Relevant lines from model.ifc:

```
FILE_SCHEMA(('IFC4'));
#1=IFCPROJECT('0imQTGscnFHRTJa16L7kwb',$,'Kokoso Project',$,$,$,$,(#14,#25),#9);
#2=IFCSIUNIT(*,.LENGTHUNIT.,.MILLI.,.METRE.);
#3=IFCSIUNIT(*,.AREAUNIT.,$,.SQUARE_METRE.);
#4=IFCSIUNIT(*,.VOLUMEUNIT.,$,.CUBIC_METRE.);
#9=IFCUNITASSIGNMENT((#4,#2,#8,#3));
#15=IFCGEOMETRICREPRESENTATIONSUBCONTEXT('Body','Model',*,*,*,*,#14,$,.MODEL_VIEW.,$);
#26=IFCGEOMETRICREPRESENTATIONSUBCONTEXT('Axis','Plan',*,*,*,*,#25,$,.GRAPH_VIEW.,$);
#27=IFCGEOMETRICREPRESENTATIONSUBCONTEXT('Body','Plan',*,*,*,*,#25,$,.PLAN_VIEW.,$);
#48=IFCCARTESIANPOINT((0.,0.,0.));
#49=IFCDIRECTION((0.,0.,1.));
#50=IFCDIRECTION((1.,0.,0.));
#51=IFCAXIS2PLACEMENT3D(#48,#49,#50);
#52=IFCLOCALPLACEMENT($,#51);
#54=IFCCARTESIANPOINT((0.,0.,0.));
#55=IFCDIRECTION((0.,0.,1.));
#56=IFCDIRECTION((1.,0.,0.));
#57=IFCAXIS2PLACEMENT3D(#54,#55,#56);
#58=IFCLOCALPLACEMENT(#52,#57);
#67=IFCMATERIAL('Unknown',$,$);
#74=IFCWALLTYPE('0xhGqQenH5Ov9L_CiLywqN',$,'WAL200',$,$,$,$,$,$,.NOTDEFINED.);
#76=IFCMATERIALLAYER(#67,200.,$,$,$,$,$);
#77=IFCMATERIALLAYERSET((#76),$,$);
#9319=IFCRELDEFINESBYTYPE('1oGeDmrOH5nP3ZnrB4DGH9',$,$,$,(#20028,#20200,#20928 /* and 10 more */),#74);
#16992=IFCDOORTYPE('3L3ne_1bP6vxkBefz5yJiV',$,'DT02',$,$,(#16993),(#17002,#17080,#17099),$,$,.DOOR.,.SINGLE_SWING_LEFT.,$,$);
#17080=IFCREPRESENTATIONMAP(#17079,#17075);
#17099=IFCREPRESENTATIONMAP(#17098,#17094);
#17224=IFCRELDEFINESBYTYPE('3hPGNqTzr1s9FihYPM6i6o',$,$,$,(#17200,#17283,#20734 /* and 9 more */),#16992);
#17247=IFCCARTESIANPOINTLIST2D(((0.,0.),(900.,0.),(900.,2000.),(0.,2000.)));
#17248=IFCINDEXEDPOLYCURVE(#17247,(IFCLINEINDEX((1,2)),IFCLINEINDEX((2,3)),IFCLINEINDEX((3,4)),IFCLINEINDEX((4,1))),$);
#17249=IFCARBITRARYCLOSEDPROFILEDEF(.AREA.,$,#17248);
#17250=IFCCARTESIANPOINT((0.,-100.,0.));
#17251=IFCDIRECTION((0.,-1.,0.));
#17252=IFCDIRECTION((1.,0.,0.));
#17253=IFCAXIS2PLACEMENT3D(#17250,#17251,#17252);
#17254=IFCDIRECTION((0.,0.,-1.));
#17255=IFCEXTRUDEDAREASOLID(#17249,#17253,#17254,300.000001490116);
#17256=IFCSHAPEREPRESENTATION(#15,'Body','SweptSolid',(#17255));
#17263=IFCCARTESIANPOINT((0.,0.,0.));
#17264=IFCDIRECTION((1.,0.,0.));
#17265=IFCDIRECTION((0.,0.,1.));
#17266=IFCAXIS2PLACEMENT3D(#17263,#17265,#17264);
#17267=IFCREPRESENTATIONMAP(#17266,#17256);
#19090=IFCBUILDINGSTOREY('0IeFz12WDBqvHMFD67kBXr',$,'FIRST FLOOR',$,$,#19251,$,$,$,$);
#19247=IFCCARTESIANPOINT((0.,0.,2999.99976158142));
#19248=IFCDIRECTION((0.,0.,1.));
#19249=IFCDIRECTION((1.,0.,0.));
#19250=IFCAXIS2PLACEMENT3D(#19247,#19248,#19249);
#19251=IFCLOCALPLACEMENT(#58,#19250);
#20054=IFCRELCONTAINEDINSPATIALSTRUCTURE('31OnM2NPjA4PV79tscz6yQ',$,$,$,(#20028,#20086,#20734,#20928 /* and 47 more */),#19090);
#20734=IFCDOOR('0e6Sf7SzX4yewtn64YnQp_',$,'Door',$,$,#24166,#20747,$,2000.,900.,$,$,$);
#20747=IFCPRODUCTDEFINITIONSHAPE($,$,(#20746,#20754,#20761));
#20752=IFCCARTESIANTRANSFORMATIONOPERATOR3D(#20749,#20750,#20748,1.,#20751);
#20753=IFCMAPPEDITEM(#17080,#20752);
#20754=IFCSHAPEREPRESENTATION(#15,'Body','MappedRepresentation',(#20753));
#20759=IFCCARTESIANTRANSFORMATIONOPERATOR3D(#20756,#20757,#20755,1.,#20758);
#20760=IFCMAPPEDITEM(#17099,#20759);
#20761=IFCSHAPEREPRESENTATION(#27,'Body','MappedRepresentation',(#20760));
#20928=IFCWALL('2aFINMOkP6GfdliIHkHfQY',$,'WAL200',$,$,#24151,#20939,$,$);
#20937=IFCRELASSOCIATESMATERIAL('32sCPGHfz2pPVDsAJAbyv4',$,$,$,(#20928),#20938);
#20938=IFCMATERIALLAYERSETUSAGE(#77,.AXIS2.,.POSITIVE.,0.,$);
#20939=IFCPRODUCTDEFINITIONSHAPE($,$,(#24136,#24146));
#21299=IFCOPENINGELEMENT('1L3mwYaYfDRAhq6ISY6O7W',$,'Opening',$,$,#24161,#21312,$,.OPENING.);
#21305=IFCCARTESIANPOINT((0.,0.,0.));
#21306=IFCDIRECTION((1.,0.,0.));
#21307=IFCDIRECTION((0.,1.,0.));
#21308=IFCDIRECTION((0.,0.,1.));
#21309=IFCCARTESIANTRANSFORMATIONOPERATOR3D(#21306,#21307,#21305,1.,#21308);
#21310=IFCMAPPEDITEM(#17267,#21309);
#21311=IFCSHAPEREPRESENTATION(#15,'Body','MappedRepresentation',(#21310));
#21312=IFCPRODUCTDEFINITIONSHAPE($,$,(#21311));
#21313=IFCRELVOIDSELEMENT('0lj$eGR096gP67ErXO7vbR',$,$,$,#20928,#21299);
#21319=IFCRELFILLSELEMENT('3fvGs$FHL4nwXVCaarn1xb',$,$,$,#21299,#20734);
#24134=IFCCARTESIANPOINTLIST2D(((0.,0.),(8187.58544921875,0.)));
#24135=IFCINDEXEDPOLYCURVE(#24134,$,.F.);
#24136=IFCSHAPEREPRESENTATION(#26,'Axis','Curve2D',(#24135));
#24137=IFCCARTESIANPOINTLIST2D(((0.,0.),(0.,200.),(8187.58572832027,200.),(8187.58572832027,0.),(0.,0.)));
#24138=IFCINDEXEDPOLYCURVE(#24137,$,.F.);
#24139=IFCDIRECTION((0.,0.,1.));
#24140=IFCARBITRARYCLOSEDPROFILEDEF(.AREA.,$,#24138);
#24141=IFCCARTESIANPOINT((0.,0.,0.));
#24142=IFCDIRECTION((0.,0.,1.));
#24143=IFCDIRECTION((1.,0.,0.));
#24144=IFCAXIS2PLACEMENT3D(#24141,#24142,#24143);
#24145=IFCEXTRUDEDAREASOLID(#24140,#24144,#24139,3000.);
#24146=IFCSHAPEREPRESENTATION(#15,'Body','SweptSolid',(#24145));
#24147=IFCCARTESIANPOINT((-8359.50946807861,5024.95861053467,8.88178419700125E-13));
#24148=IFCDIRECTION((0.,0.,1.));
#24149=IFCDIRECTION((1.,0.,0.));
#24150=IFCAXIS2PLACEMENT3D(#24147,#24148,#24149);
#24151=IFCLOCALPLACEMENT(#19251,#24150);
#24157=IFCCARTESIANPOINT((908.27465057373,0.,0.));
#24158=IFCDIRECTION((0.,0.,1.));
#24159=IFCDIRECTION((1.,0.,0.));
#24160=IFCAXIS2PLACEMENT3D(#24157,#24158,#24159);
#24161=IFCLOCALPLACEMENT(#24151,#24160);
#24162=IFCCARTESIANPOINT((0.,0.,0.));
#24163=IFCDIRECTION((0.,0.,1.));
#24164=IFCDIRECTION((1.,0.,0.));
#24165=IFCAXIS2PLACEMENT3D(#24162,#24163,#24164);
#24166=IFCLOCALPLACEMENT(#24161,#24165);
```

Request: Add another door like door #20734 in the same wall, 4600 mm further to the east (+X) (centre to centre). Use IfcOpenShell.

```python
import ifcopenshell
import ifcopenshell.api.feature
import ifcopenshell.api.geometry
import ifcopenshell.api.root
import ifcopenshell.geom
import ifcopenshell.util.element
import ifcopenshell.util.placement
import ifcopenshell.util.shape
import ifcopenshell.util.unit

model = ifcopenshell.open("model.ifc")
unit_scale = ifcopenshell.util.unit.calculate_unit_scale(model)
settings = ifcopenshell.geom.settings()


def volume(element):
    """Net volume in cubic metres, openings subtracted."""
    shape = ifcopenshell.geom.create_shape(settings, element)
    return ifcopenshell.util.shape.get_volume(shape.geometry)


door = model.by_guid("0e6Sf7SzX4yewtn64YnQp_")
opening = door.FillsVoids[0].RelatingOpeningElement
wall = opening.VoidsElements[0].RelatingBuildingElement
before = volume(wall)
shift = ifcopenshell.util.placement.get_local_placement(wall.ObjectPlacement)[:3, 0] * 4.6 / unit_scale

# copy_class copies the void relationship, type, container and properties, but no geometry.
new_opening = ifcopenshell.api.root.copy_class(model, product=opening)
new_opening.Representation = ifcopenshell.util.element.copy_deep(
    model, opening.Representation, exclude=["IfcGeometricRepresentationContext", "IfcRepresentationMap"]
)
new_door = ifcopenshell.api.root.copy_class(model, product=door)
new_door.Representation = ifcopenshell.util.element.copy_deep(
    model, door.Representation, exclude=["IfcGeometricRepresentationContext", "IfcRepresentationMap"]
)
ifcopenshell.api.feature.add_filling(model, opening=new_opening, element=new_door)

for old, new in ((opening, new_opening), (door, new_door)):
    matrix = ifcopenshell.util.placement.get_local_placement(old.ObjectPlacement)
    matrix[:3, 3] += shift
    ifcopenshell.api.geometry.edit_object_placement(model, product=new, matrix=matrix, is_si=False)

after = volume(wall)

print(f"wall volume {before:.3f} -> {after:.3f} m3")

model.write("model_v2.ifc")
```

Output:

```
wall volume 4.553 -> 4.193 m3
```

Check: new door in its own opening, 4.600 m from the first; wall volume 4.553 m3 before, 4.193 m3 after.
